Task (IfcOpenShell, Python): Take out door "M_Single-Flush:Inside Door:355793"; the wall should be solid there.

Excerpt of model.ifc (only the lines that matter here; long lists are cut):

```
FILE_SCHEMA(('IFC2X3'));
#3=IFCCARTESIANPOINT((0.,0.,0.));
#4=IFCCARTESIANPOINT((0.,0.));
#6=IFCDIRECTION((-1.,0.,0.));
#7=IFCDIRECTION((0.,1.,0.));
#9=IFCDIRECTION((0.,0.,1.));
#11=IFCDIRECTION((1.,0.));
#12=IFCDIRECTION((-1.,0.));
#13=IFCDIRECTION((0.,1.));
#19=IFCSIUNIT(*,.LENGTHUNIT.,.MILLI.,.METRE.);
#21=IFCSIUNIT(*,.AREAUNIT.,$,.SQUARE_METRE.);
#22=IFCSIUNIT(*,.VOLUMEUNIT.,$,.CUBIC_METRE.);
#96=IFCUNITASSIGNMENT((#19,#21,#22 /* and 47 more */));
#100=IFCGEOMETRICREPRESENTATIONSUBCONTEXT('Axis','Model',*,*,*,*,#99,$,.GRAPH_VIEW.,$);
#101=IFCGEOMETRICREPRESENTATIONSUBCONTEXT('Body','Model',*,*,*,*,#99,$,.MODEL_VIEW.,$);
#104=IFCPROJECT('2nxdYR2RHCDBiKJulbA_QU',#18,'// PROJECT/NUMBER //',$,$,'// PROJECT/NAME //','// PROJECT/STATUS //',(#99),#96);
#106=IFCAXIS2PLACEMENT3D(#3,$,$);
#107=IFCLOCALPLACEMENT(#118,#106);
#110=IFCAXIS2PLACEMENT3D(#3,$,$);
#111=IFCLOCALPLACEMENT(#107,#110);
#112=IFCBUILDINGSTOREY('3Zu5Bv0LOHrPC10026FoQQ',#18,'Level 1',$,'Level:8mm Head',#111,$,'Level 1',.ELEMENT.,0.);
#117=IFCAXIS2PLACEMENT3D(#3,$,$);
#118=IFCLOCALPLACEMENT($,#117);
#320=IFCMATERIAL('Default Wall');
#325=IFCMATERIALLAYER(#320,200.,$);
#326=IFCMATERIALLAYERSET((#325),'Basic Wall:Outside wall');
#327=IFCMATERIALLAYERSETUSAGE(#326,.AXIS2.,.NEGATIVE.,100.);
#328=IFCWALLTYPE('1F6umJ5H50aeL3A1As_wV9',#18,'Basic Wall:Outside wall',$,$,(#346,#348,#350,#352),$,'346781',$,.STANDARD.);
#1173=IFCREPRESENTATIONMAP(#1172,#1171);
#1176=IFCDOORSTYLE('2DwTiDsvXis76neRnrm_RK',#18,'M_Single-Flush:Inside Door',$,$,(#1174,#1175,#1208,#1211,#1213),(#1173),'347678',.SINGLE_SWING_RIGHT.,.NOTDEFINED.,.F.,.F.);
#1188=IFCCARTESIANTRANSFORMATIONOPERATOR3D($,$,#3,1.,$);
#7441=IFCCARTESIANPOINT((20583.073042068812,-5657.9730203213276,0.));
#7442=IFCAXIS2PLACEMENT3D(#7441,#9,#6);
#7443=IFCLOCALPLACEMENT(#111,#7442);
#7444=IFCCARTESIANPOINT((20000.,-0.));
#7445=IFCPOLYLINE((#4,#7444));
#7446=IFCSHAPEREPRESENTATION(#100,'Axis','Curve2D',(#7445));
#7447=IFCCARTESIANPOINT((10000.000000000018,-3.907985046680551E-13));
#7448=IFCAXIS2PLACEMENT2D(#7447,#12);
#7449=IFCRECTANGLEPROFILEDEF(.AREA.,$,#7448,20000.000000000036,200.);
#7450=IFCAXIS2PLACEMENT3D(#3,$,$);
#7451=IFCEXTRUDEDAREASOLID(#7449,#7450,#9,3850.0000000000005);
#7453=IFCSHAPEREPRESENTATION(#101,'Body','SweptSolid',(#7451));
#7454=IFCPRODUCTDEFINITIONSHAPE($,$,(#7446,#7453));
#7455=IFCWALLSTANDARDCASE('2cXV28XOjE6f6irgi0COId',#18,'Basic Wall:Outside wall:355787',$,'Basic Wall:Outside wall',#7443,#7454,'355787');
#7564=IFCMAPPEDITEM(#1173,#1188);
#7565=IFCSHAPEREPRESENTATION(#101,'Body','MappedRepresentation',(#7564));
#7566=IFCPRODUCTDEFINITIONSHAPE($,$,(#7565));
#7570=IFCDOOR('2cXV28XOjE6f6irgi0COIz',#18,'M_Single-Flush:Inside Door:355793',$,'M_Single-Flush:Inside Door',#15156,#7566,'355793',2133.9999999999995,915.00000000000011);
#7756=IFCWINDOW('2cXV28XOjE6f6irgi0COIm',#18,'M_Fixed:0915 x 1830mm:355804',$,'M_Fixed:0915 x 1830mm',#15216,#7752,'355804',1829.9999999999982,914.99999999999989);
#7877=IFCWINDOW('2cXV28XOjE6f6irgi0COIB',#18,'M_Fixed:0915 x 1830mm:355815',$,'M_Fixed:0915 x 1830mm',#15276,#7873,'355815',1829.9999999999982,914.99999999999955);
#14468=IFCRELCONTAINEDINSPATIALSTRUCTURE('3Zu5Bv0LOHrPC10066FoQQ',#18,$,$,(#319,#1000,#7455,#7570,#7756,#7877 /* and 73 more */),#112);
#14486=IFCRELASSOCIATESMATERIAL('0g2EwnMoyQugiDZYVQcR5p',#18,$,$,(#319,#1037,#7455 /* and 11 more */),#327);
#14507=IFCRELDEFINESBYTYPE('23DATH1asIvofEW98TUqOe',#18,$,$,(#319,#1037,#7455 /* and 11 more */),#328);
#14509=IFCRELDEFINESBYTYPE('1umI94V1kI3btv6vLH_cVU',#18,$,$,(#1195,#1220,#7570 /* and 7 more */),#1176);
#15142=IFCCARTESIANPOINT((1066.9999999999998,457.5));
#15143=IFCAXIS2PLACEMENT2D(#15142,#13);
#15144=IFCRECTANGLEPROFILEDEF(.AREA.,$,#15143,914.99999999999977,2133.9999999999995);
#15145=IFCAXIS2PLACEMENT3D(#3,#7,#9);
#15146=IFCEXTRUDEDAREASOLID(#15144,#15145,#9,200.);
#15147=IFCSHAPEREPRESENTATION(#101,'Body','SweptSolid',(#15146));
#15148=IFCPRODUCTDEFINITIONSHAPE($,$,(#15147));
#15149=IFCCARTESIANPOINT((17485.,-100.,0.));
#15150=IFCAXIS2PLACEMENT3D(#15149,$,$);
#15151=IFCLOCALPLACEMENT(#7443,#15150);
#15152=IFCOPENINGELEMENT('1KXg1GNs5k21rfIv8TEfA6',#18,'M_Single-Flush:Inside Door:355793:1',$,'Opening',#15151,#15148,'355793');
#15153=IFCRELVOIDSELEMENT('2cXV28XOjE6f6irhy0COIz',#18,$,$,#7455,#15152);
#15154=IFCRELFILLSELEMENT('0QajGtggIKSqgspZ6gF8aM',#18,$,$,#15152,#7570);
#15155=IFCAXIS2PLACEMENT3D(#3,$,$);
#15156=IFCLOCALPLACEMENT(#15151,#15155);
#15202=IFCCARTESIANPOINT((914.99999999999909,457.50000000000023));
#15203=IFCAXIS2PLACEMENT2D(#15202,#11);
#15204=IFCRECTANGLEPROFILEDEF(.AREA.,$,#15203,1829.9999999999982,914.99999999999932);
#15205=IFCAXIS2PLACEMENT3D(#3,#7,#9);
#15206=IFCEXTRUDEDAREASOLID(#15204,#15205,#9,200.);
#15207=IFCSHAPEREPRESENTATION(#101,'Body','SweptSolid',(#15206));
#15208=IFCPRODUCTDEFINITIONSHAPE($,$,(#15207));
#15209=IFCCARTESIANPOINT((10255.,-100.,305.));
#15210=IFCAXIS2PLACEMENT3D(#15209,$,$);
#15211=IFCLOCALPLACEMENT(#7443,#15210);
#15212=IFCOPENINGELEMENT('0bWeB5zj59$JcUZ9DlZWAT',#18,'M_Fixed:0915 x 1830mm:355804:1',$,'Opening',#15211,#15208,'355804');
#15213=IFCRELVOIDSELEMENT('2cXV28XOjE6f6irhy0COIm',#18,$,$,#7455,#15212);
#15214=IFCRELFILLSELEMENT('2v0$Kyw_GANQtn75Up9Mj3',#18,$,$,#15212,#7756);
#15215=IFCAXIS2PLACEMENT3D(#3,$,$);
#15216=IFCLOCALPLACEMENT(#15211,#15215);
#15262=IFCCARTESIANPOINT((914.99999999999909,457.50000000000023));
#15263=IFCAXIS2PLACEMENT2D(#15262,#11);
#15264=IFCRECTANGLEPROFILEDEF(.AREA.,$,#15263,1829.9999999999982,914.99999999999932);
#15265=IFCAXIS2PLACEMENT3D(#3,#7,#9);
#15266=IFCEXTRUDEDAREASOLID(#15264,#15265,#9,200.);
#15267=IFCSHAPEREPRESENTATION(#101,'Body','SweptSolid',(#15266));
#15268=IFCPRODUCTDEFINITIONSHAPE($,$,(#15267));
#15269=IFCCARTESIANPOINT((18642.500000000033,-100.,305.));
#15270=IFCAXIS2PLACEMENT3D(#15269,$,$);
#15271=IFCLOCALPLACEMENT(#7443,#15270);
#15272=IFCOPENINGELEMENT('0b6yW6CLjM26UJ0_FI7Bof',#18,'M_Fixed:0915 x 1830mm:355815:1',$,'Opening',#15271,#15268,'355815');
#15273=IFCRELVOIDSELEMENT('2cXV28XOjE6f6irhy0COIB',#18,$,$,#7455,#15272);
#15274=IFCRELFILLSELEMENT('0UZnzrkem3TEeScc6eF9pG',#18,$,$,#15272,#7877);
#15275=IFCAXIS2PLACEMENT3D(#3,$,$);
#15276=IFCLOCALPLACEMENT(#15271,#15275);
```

```python
import ifcopenshell
import ifcopenshell.api.feature
import ifcopenshell.api.root
import ifcopenshell.geom
import ifcopenshell.util.shape

model = ifcopenshell.open("model.ifc")
settings = ifcopenshell.geom.settings()


def volume(element):
    """Net volume in cubic metres, openings subtracted."""
    shape = ifcopenshell.geom.create_shape(settings, element)
    return ifcopenshell.util.shape.get_volume(shape.geometry)


door = model.by_guid("2cXV28XOjE6f6irgi0COIz")
opening = door.FillsVoids[0].RelatingOpeningElement
wall = opening.VoidsElements[0].RelatingBuildingElement
before = volume(wall)

ifcopenshell.api.root.remove_product(model, product=door)
ifcopenshell.api.feature.remove_feature(model, feature=opening)

after = volume(wall)

print(f"wall volume {before:.3f} -> {after:.3f} m3")

model.write("model_v2.ifc")
```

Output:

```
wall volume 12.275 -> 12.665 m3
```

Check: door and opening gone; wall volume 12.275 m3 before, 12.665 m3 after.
